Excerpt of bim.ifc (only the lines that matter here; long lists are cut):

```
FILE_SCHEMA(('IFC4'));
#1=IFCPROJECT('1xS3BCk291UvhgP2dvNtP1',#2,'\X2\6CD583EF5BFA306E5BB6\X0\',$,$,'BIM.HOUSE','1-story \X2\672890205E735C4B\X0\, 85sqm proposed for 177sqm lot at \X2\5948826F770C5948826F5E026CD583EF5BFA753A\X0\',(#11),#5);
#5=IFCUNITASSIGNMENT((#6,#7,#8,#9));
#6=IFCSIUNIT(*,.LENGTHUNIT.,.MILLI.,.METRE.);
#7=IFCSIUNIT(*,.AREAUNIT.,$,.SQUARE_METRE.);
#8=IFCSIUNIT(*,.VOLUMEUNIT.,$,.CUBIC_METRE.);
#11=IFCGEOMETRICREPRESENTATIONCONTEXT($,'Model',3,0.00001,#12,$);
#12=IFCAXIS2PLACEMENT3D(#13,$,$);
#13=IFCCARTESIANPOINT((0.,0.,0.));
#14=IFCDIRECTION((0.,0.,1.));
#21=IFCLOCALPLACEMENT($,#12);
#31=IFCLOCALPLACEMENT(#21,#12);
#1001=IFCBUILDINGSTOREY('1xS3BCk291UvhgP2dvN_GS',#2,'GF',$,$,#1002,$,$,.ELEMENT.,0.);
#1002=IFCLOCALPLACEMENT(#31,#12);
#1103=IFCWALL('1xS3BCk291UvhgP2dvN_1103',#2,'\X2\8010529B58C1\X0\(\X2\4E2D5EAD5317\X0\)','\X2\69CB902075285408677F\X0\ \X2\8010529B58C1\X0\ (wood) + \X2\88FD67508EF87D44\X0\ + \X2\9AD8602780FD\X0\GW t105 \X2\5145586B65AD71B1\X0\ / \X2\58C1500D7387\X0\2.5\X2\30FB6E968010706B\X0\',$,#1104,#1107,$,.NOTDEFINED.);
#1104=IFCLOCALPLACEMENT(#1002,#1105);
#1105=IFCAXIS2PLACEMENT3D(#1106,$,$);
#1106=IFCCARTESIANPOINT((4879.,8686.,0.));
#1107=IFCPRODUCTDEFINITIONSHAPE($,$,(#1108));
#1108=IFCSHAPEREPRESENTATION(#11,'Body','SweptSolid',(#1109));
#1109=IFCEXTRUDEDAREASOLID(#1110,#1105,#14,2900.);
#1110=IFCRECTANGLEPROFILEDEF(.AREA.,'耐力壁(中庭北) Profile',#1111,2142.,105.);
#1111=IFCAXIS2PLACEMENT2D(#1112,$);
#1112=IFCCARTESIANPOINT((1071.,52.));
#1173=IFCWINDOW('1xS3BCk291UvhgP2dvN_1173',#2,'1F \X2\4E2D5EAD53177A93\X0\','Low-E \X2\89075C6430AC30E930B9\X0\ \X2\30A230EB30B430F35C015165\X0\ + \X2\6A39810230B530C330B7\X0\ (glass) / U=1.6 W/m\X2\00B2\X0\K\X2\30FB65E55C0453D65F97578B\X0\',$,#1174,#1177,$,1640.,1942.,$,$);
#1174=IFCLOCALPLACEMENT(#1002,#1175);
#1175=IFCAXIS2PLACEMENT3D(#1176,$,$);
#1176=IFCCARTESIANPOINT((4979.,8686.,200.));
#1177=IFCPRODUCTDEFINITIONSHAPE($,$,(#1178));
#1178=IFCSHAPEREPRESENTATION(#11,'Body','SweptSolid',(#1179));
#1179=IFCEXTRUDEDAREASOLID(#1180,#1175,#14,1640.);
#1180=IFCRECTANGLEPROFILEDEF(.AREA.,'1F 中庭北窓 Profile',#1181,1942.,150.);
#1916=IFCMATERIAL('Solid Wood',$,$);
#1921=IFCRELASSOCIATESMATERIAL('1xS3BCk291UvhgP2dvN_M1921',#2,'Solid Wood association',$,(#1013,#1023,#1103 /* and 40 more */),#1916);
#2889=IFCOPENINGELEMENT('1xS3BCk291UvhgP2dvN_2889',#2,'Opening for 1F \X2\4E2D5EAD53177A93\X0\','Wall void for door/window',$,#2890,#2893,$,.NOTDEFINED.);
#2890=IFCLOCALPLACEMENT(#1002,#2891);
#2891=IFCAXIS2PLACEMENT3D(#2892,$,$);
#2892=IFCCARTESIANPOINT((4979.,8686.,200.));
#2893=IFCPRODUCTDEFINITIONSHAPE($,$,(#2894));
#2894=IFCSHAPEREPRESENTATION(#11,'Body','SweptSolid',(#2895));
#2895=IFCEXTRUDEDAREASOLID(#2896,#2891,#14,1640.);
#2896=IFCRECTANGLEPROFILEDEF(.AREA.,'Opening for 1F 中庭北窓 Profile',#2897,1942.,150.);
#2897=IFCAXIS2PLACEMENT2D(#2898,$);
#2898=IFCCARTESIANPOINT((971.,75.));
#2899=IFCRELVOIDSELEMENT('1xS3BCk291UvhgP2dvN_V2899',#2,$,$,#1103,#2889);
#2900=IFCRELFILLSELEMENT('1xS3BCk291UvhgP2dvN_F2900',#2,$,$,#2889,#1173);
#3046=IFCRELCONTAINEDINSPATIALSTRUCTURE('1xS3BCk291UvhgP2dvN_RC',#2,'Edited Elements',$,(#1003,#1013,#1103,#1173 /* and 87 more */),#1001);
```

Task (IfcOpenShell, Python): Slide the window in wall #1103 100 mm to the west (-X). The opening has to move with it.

```python
import ifcopenshell
import ifcopenshell.api.geometry
import ifcopenshell.util.placement
import ifcopenshell.util.unit

model = ifcopenshell.open("bim.ifc")
unit_scale = ifcopenshell.util.unit.calculate_unit_scale(model)

window = model.by_guid("1xS3BCk291UvhgP2dvN_1173")
opening = window.FillsVoids[0].RelatingOpeningElement
wall = opening.VoidsElements[0].RelatingBuildingElement

wall_matrix = ifcopenshell.util.placement.get_local_placement(wall.ObjectPlacement)
shift = wall_matrix[:3, 0] * -0.1 / unit_scale
before = ifcopenshell.util.placement.get_local_placement(window.ObjectPlacement)[:3, 3].copy()

# The window is not placed relative to its opening, so move both.
for product in (opening, window):
    matrix = ifcopenshell.util.placement.get_local_placement(product.ObjectPlacement)
    matrix[:3, 3] += shift
    ifcopenshell.api.geometry.edit_object_placement(model, product=product, matrix=matrix, is_si=False)

after = ifcopenshell.util.placement.get_local_placement(window.ObjectPlacement)[:3, 3]
print("window moved by", (after - before).round(3) + 0.0)

model.write("bim_updated.ifc")
```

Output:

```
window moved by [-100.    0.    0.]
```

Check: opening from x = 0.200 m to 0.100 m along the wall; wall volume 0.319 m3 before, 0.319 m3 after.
